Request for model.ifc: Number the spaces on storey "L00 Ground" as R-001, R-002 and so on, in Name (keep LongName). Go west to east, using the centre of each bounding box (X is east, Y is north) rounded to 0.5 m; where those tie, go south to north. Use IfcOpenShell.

First a look at what the model holds.

```python
import ifcopenshell
import ifcopenshell.util.element
import ifcopenshell.util.placement

model = ifcopenshell.open("model.ifc")
print(model.schema)
storey = next(s for s in model.by_type("IfcBuildingStorey") if s.Name == "L00 Ground")
spaces = [e for e in ifcopenshell.util.element.get_decomposition(storey) if e.is_a("IfcSpace")]
for e in sorted(spaces, key=lambda e: e.id()):
    origin = ifcopenshell.util.placement.get_local_placement(e.ObjectPlacement)[:3, 3]
    print(e.id(), e.Name, e.LongName, origin.round(2) + 0.0, sep=" | ")
```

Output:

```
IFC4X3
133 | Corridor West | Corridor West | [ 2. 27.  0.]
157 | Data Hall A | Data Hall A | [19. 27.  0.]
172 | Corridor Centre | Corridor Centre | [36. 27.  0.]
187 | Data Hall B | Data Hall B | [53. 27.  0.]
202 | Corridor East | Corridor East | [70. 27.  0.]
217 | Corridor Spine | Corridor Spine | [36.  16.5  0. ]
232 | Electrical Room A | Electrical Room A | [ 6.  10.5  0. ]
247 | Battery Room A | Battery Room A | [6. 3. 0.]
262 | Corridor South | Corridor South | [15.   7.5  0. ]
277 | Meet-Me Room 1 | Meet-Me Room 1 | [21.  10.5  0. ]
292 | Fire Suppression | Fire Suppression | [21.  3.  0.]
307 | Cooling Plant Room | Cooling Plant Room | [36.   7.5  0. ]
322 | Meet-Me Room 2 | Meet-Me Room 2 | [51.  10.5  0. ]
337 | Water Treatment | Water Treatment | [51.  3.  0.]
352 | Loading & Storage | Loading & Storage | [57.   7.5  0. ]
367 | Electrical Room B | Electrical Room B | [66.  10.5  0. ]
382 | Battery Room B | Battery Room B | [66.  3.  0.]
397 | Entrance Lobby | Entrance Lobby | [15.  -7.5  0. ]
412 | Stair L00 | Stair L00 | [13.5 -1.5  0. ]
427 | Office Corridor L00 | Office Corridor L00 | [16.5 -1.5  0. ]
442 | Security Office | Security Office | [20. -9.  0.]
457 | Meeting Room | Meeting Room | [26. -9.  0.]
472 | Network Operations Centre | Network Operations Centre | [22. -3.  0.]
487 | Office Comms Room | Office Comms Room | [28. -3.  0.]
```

```python
import ifcopenshell
import ifcopenshell.geom
import ifcopenshell.util.element
import ifcopenshell.util.shape

model = ifcopenshell.open("model.ifc")
settings = ifcopenshell.geom.settings()
settings.set("use-world-coords", True)


def centre(element):
    shape = ifcopenshell.geom.create_shape(settings, element)
    return ifcopenshell.util.shape.get_bbox_centroid(shape.geometry)


storey = next(s for s in model.by_type("IfcBuildingStorey") if s.Name == "L00 Ground")
spaces = [e for e in ifcopenshell.util.element.get_decomposition(storey) if e.is_a("IfcSpace")]

# Insertion points can sit at a corner or the storey origin, so sort by the geometry (in metres).
centres = {e: centre(e) for e in spaces}
spaces.sort(key=lambda e: (round(centres[e][0] / 0.5), centres[e][1]))

for i, e in enumerate(spaces, start=1):
    number = f"R-0{i:02d}"
    e.Name = number
    print(e.id(), number)

model.write("model_v2.ifc")
```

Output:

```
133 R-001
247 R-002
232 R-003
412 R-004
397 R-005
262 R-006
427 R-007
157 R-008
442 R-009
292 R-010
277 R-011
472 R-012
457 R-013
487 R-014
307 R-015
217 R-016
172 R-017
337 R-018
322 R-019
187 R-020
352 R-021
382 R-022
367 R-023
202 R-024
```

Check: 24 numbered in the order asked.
